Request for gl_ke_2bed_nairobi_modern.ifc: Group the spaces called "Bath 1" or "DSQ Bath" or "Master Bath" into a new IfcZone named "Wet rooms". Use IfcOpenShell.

First a look at what the model holds.

```python
import ifcopenshell

model = ifcopenshell.open("gl_ke_2bed_nairobi_modern.ifc")
print(model.schema)
seen = {}
for space in model.by_type("IfcSpace"):
    seen[space.LongName] = seen.get(space.LongName, 0) + 1
for name, count in sorted(seen.items(), key=str):
    print(count, "x", name)
print("zones:", [z.Name for z in model.by_type("IfcZone")][:20])
```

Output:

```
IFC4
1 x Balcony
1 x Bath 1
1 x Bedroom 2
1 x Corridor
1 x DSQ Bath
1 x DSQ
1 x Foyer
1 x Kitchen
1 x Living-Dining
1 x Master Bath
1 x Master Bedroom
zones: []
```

```python
import ifcopenshell
import ifcopenshell.api.group
import ifcopenshell.api.root

model = ifcopenshell.open("gl_ke_2bed_nairobi_modern.ifc")

names = {"Bath 1", "DSQ Bath", "Master Bath"}
spaces = [s for s in model.by_type("IfcSpace") if s.LongName in names]

zone = ifcopenshell.api.root.create_entity(model, ifc_class="IfcZone", name="Wet rooms")
ifcopenshell.api.group.assign_group(model, products=spaces, group=zone)
print(len(spaces), "spaces in", zone.Name)

model.write("gl_ke_2bed_nairobi_modern_updated.ifc")
```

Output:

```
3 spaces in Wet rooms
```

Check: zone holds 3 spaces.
